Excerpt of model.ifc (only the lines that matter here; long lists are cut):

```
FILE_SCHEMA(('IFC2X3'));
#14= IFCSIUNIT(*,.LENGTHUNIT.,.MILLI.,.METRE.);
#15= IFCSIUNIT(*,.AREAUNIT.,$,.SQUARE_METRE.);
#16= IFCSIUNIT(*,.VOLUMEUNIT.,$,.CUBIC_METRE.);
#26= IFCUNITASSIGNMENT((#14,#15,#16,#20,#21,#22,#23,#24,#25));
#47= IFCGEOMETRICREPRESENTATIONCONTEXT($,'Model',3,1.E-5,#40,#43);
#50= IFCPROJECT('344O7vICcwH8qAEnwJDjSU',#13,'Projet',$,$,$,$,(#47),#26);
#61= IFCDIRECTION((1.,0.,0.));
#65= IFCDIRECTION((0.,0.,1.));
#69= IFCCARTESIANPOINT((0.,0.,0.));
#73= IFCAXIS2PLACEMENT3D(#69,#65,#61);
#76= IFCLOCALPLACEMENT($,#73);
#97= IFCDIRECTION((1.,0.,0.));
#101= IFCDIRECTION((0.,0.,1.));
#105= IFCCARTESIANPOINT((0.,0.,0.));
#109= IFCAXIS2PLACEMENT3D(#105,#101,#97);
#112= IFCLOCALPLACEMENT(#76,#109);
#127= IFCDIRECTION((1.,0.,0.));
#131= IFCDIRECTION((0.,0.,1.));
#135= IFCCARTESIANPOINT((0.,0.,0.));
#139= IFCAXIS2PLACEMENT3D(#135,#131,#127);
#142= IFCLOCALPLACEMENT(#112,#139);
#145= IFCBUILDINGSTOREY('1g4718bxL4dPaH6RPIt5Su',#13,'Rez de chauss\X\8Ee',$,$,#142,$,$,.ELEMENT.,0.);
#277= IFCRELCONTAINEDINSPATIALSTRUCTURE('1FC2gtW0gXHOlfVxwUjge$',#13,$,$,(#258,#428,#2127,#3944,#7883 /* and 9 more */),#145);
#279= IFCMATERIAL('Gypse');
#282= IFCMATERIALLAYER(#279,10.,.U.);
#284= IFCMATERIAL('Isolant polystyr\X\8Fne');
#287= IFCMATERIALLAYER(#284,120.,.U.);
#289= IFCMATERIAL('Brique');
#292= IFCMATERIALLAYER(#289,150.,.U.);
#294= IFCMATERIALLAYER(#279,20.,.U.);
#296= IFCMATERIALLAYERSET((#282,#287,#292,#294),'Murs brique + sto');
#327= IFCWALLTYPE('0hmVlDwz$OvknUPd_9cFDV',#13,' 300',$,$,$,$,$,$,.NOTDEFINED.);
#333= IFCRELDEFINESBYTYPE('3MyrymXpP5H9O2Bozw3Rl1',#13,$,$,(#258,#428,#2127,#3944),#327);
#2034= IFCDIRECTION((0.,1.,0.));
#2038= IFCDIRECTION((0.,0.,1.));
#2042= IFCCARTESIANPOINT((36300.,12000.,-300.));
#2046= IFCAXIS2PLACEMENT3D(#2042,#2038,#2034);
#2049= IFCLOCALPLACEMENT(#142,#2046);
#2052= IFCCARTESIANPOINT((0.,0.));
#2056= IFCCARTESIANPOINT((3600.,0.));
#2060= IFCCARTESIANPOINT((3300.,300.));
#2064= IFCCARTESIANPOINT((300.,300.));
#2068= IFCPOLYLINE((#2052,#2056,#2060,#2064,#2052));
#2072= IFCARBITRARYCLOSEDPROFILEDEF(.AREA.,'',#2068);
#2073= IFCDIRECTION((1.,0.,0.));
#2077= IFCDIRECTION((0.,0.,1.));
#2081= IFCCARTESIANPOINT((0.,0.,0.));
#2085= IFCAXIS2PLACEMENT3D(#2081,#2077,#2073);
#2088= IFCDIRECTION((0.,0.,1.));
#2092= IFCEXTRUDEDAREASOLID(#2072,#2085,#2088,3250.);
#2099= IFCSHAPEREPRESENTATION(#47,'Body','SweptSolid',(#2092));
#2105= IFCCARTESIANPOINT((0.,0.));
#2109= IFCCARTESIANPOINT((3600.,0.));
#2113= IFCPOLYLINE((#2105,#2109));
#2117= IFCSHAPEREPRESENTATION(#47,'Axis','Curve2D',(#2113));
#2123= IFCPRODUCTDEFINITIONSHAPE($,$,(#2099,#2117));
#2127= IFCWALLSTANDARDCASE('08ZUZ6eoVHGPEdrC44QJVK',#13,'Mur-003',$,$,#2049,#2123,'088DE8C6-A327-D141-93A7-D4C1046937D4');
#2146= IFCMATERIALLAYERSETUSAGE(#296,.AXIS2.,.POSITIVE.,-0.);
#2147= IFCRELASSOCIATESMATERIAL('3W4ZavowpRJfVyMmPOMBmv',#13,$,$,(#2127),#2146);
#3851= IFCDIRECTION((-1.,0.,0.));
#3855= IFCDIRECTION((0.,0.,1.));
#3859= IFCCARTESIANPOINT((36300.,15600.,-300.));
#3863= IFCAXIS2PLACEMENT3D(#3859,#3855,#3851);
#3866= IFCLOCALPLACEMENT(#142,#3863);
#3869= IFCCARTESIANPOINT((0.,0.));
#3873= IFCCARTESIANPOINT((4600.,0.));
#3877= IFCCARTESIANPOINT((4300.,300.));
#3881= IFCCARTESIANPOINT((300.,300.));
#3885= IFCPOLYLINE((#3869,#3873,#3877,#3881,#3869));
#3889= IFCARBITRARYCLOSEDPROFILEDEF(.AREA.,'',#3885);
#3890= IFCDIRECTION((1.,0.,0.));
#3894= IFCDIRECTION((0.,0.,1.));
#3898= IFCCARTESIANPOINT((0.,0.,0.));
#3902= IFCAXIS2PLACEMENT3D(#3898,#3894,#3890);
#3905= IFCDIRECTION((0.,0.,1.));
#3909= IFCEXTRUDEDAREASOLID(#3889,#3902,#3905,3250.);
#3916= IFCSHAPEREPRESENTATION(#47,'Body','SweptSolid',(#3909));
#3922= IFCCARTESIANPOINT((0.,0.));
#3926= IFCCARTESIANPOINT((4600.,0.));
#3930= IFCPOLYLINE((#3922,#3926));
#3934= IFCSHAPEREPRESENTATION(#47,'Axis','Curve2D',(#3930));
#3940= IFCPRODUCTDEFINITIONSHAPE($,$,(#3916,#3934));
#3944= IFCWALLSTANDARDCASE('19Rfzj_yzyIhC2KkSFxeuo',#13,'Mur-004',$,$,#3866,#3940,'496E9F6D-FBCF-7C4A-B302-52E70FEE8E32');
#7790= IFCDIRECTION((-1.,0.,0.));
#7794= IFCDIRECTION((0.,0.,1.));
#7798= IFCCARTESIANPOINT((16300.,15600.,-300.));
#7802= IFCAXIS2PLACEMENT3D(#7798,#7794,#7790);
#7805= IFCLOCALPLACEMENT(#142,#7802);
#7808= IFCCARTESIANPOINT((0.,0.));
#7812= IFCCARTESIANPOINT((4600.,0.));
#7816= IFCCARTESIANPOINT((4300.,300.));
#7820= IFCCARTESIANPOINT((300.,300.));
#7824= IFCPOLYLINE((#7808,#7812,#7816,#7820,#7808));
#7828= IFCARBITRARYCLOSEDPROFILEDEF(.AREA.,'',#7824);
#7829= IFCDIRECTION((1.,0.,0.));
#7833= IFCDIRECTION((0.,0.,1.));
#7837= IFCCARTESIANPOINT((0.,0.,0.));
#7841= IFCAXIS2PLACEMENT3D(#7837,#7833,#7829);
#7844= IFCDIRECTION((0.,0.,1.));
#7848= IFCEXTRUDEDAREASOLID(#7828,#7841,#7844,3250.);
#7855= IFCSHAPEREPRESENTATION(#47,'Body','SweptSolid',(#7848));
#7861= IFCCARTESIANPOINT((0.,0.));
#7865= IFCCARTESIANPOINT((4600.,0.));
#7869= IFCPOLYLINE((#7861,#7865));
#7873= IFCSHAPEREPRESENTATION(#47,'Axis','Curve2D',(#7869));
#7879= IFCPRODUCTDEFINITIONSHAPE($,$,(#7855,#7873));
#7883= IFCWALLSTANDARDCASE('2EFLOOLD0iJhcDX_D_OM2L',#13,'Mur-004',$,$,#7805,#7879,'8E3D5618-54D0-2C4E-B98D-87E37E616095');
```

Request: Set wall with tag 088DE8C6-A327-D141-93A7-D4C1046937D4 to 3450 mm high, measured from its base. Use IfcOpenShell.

```python
import ifcopenshell
import ifcopenshell.geom
import ifcopenshell.util.shape
import ifcopenshell.util.unit

model = ifcopenshell.open("model.ifc")
unit_scale = ifcopenshell.util.unit.calculate_unit_scale(model)
settings = ifcopenshell.geom.settings()


def volume(element):
    """Net volume in cubic metres, openings subtracted."""
    shape = ifcopenshell.geom.create_shape(settings, element)
    return ifcopenshell.util.shape.get_volume(shape.geometry)


wall = model.by_guid("08ZUZ6eoVHGPEdrC44QJVK")
before = volume(wall)

body = next(r for r in wall.Representation.Representations if r.RepresentationIdentifier == "Body")
solid = body.Items[0]
old_height = solid.Depth
solid.Depth = 3.45 / unit_scale
after = volume(wall)

print(f"height {old_height:g} -> {solid.Depth:g}, volume {before:.3f} -> {after:.3f} m3")

model.write("model_updated.ifc")
```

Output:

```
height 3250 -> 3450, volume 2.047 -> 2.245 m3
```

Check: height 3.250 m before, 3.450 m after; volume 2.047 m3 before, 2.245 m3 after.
